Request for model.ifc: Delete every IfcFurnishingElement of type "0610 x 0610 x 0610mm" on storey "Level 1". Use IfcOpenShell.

First a look at what the model holds.

```python
import ifcopenshell
import ifcopenshell.util.element

model = ifcopenshell.open("model.ifc")
print(model.schema)
storey = next(s for s in model.by_type("IfcBuildingStorey") if s.Name == "Level 1")
furniture = [e for e in ifcopenshell.util.element.get_decomposition(storey) if e.is_a("IfcFurnishingElement")]
seen = {}
for e in furniture:
    element_type = ifcopenshell.util.element.get_type(e)
    name = element_type.Name if element_type not in (None, e) else None
    seen[name] = seen.get(name, 0) + 1
for name, count in sorted(seen.items(), key=str):
    print(count, "x", name)
```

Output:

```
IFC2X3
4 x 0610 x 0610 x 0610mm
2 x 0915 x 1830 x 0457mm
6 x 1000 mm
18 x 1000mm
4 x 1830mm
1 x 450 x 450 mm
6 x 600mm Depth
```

```python
import ifcopenshell
import ifcopenshell.api.root
import ifcopenshell.util.element

model = ifcopenshell.open("model.ifc")

storey = next(s for s in model.by_type("IfcBuildingStorey") if s.Name == "Level 1")
furniture = [e for e in ifcopenshell.util.element.get_decomposition(storey) if e.is_a("IfcFurnishingElement")]
targets = [e for e in furniture if (t := ifcopenshell.util.element.get_type(e)) not in (None, e) and t.Name == "0610 x 0610 x 0610mm"]

for e in targets:
    ifcopenshell.api.root.remove_product(model, product=e)
print(len(targets), "removed")

model.write("model_updated.ifc")
```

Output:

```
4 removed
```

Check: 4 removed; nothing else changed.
